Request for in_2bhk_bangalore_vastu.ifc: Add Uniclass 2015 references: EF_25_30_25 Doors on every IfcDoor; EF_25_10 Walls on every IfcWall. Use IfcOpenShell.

First a look at what the model holds.

```python
import ifcopenshell

model = ifcopenshell.open("in_2bhk_bangalore_vastu.ifc")
print(model.schema)
print("classifications:", [c.Name for c in model.by_type("IfcClassification")])
for ifc_class in ("IfcDoor", "IfcRoof", "IfcStair", "IfcWall", "IfcWindow"):
    print(ifc_class, len(model.by_type(ifc_class)))
```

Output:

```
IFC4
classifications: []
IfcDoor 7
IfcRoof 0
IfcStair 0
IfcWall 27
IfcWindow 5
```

```python
import ifcopenshell
import ifcopenshell.api.classification

model = ifcopenshell.open("in_2bhk_bangalore_vastu.ifc")

system = ifcopenshell.api.classification.add_classification(model, classification="Uniclass 2015")

codes = {
    "IfcDoor": ("EF_25_30_25", "Doors"),
    "IfcWall": ("EF_25_10", "Walls"),
}
for ifc_class, (code, name) in codes.items():
    products = model.by_type(ifc_class)
    ifcopenshell.api.classification.add_reference(
        model, products=products, classification=system, identification=code, name=name
    )
    print(code, len(products))

model.write("in_2bhk_bangalore_vastu_rev.ifc")
```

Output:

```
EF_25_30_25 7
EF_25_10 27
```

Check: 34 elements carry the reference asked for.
